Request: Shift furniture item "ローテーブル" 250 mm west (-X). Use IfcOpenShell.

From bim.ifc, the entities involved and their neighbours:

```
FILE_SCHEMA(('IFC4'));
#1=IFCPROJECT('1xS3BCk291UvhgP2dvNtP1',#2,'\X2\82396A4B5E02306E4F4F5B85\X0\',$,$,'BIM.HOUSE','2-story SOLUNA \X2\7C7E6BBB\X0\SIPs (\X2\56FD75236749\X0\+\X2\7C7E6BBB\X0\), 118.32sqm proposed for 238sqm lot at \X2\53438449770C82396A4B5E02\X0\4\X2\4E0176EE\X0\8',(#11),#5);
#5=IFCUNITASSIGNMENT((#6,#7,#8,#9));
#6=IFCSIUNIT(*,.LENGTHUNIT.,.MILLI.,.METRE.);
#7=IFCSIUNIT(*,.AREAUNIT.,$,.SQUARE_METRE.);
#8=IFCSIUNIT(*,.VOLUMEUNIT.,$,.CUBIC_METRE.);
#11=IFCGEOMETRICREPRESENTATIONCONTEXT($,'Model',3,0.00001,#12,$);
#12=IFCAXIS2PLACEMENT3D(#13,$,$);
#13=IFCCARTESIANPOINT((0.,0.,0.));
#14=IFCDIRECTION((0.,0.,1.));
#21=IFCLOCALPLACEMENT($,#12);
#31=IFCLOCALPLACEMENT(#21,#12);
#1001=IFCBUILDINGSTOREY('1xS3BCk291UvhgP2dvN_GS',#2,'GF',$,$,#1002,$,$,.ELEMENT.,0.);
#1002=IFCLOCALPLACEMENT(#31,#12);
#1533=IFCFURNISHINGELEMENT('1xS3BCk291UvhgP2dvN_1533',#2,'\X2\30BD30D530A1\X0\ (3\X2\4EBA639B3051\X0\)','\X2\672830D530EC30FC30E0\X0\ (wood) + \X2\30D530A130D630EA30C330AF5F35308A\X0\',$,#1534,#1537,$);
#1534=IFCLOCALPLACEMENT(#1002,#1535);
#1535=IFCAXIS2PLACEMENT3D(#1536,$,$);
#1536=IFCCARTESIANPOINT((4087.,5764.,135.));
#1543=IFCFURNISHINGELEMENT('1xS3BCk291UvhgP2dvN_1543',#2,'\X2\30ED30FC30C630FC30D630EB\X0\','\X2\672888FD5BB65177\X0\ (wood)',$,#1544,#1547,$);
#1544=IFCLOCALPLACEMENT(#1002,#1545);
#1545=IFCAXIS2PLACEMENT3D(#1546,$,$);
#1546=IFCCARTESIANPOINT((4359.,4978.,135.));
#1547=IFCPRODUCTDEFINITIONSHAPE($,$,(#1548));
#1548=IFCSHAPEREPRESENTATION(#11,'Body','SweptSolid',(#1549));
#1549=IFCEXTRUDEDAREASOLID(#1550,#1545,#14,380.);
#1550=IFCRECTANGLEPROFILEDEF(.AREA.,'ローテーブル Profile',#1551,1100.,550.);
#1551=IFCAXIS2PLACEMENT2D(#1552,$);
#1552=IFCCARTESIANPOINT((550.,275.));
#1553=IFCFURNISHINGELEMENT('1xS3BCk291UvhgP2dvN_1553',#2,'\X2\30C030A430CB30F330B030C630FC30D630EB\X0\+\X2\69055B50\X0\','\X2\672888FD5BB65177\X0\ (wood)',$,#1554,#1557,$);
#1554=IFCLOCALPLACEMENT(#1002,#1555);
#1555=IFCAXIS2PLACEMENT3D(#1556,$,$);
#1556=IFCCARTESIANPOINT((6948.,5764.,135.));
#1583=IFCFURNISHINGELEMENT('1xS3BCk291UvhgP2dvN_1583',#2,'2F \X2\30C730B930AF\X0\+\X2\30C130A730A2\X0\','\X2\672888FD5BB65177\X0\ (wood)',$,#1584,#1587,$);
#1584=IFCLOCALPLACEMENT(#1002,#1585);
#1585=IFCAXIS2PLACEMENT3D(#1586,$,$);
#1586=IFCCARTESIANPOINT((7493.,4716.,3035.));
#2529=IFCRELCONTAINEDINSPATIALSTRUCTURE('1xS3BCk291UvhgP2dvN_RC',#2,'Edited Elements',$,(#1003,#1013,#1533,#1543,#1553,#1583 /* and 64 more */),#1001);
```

```python
import ifcopenshell
import ifcopenshell.api.geometry
import ifcopenshell.util.placement

model = ifcopenshell.open("bim.ifc")

item = model.by_guid("1xS3BCk291UvhgP2dvN_1543")
matrix = ifcopenshell.util.placement.get_local_placement(item.ObjectPlacement)
matrix[0, 3] -= 250.0
ifcopenshell.api.geometry.edit_object_placement(model, product=item, matrix=matrix, is_si=False)

print(ifcopenshell.util.placement.get_local_placement(item.ObjectPlacement).round(3) + 0.0)

model.write("bim_rev.ifc")
```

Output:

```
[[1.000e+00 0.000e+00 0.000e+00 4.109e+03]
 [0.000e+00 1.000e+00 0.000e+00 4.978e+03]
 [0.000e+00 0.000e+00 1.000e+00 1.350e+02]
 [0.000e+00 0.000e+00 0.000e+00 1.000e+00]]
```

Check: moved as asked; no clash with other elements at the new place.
